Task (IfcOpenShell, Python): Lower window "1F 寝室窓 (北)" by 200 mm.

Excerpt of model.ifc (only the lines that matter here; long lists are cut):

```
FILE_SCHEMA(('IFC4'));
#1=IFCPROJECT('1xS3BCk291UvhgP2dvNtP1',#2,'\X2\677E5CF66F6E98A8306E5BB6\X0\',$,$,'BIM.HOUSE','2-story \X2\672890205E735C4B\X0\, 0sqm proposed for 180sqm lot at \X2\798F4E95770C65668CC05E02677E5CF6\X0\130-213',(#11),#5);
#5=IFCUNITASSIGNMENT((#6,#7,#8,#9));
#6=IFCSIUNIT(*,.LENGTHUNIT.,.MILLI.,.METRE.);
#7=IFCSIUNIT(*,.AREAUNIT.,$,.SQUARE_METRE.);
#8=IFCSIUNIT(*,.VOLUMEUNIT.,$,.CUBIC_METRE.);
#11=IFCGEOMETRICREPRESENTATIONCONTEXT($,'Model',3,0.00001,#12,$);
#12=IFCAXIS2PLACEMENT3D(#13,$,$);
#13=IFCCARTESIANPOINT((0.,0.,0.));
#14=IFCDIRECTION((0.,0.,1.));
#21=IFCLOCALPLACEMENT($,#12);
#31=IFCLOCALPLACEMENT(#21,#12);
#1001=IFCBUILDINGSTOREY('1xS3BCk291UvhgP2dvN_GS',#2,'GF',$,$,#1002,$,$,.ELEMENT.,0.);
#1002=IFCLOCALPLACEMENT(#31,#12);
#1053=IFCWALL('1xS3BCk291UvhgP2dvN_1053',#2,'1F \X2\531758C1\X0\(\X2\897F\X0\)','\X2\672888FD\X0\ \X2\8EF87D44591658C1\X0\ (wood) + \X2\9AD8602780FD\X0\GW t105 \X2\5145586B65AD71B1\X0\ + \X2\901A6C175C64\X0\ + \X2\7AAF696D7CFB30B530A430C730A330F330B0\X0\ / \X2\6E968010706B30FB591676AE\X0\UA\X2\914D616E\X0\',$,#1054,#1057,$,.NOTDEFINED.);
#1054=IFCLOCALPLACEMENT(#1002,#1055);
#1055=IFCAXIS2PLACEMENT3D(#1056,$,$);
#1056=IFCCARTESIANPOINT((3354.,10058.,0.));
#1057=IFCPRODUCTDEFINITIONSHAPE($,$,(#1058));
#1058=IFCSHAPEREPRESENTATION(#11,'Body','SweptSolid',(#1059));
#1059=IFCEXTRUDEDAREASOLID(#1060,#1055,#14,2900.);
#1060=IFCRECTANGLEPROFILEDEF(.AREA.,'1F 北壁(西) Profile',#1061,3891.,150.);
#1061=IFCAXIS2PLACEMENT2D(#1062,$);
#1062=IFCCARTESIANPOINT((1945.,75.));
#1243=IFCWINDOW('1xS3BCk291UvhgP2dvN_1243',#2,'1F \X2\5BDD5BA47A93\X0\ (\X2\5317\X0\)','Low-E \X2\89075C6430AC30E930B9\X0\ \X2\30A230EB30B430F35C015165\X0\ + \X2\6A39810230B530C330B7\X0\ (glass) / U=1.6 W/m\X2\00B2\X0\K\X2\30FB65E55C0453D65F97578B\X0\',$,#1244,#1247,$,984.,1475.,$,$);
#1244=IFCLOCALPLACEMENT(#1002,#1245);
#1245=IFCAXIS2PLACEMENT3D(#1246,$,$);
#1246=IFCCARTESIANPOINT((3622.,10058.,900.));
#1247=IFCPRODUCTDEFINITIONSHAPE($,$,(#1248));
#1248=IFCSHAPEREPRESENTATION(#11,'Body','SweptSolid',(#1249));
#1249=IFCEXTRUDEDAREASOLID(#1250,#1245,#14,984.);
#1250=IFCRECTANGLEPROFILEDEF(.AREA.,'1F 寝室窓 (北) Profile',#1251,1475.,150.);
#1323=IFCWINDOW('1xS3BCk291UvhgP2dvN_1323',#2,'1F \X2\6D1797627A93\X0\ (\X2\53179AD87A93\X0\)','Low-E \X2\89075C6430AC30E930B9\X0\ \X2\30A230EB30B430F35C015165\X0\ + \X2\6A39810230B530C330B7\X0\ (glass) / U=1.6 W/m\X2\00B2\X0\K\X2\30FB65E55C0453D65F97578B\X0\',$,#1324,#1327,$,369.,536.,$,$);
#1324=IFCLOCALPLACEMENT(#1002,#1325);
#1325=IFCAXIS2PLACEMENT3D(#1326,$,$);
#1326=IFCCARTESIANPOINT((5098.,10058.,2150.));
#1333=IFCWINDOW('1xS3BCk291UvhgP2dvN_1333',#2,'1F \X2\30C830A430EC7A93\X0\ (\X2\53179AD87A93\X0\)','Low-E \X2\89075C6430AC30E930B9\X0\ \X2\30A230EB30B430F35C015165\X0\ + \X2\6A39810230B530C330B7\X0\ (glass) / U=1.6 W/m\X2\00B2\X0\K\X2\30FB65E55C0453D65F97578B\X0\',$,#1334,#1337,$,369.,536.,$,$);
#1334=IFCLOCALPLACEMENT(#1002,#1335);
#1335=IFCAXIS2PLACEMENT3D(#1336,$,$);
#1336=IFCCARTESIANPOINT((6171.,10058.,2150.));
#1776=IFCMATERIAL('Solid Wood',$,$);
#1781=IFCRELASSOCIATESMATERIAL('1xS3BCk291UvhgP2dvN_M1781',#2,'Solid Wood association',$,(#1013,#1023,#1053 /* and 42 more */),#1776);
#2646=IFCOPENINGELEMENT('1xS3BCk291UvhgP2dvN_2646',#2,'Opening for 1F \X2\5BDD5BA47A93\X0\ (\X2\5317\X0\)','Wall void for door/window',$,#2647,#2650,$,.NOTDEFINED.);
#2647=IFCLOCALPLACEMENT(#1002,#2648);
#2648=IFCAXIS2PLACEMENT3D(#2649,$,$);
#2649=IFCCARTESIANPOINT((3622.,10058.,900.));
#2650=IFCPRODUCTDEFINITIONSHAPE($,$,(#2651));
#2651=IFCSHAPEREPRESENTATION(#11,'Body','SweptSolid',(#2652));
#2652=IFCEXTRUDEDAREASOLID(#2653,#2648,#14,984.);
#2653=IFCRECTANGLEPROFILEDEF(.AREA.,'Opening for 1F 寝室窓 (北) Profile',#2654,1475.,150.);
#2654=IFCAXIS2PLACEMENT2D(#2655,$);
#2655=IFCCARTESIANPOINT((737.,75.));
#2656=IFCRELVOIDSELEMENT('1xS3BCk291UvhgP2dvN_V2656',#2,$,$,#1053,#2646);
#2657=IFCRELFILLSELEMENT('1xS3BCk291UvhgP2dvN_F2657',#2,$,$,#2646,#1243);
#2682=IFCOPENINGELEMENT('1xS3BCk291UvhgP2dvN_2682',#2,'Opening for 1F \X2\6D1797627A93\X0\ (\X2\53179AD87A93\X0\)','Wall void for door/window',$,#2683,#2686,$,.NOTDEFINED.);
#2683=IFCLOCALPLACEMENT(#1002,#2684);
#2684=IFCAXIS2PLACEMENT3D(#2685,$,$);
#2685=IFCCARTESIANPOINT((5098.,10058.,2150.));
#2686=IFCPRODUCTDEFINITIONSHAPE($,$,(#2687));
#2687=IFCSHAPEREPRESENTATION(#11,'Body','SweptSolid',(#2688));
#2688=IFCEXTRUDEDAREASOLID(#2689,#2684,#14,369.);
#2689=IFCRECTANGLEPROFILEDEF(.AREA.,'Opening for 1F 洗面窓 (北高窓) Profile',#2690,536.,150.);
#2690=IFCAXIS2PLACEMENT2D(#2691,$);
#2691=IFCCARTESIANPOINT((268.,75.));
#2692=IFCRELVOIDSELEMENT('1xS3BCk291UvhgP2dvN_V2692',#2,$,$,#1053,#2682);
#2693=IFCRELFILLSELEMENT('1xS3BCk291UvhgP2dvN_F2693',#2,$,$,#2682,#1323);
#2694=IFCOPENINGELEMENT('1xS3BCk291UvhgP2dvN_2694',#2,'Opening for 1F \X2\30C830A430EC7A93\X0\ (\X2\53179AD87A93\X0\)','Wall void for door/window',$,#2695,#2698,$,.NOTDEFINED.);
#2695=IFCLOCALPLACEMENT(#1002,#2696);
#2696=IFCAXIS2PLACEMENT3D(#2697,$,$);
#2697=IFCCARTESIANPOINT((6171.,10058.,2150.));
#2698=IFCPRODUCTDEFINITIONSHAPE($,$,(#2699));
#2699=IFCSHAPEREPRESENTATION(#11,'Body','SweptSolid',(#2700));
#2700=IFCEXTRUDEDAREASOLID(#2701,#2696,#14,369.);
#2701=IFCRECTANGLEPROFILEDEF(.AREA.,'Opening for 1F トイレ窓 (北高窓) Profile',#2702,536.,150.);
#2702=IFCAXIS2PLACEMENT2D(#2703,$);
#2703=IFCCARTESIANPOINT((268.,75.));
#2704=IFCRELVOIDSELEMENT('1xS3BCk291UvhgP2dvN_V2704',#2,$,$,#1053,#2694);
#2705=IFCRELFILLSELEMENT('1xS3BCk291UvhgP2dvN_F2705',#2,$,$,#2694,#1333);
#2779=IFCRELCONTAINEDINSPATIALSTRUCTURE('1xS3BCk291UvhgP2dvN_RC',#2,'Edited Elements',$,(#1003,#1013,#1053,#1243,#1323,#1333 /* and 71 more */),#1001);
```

```python
import numpy as np
import ifcopenshell
import ifcopenshell.api.geometry
import ifcopenshell.util.placement
import ifcopenshell.util.unit

model = ifcopenshell.open("model.ifc")
unit_scale = ifcopenshell.util.unit.calculate_unit_scale(model)

window = model.by_guid("1xS3BCk291UvhgP2dvN_1243")
opening = window.FillsVoids[0].RelatingOpeningElement
dz = -200.0

shift = np.array([0.0, 0.0, dz])
# The window is not placed relative to its opening, so move both.
for product in (opening, window):
    matrix = ifcopenshell.util.placement.get_local_placement(product.ObjectPlacement)
    matrix[:3, 3] += shift
    ifcopenshell.api.geometry.edit_object_placement(model, product=product, matrix=matrix, is_si=False)

print(f"moved by {dz * unit_scale:+.3f} m")

model.write("model_v2.ifc")
```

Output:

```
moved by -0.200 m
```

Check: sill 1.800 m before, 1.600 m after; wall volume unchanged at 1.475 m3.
